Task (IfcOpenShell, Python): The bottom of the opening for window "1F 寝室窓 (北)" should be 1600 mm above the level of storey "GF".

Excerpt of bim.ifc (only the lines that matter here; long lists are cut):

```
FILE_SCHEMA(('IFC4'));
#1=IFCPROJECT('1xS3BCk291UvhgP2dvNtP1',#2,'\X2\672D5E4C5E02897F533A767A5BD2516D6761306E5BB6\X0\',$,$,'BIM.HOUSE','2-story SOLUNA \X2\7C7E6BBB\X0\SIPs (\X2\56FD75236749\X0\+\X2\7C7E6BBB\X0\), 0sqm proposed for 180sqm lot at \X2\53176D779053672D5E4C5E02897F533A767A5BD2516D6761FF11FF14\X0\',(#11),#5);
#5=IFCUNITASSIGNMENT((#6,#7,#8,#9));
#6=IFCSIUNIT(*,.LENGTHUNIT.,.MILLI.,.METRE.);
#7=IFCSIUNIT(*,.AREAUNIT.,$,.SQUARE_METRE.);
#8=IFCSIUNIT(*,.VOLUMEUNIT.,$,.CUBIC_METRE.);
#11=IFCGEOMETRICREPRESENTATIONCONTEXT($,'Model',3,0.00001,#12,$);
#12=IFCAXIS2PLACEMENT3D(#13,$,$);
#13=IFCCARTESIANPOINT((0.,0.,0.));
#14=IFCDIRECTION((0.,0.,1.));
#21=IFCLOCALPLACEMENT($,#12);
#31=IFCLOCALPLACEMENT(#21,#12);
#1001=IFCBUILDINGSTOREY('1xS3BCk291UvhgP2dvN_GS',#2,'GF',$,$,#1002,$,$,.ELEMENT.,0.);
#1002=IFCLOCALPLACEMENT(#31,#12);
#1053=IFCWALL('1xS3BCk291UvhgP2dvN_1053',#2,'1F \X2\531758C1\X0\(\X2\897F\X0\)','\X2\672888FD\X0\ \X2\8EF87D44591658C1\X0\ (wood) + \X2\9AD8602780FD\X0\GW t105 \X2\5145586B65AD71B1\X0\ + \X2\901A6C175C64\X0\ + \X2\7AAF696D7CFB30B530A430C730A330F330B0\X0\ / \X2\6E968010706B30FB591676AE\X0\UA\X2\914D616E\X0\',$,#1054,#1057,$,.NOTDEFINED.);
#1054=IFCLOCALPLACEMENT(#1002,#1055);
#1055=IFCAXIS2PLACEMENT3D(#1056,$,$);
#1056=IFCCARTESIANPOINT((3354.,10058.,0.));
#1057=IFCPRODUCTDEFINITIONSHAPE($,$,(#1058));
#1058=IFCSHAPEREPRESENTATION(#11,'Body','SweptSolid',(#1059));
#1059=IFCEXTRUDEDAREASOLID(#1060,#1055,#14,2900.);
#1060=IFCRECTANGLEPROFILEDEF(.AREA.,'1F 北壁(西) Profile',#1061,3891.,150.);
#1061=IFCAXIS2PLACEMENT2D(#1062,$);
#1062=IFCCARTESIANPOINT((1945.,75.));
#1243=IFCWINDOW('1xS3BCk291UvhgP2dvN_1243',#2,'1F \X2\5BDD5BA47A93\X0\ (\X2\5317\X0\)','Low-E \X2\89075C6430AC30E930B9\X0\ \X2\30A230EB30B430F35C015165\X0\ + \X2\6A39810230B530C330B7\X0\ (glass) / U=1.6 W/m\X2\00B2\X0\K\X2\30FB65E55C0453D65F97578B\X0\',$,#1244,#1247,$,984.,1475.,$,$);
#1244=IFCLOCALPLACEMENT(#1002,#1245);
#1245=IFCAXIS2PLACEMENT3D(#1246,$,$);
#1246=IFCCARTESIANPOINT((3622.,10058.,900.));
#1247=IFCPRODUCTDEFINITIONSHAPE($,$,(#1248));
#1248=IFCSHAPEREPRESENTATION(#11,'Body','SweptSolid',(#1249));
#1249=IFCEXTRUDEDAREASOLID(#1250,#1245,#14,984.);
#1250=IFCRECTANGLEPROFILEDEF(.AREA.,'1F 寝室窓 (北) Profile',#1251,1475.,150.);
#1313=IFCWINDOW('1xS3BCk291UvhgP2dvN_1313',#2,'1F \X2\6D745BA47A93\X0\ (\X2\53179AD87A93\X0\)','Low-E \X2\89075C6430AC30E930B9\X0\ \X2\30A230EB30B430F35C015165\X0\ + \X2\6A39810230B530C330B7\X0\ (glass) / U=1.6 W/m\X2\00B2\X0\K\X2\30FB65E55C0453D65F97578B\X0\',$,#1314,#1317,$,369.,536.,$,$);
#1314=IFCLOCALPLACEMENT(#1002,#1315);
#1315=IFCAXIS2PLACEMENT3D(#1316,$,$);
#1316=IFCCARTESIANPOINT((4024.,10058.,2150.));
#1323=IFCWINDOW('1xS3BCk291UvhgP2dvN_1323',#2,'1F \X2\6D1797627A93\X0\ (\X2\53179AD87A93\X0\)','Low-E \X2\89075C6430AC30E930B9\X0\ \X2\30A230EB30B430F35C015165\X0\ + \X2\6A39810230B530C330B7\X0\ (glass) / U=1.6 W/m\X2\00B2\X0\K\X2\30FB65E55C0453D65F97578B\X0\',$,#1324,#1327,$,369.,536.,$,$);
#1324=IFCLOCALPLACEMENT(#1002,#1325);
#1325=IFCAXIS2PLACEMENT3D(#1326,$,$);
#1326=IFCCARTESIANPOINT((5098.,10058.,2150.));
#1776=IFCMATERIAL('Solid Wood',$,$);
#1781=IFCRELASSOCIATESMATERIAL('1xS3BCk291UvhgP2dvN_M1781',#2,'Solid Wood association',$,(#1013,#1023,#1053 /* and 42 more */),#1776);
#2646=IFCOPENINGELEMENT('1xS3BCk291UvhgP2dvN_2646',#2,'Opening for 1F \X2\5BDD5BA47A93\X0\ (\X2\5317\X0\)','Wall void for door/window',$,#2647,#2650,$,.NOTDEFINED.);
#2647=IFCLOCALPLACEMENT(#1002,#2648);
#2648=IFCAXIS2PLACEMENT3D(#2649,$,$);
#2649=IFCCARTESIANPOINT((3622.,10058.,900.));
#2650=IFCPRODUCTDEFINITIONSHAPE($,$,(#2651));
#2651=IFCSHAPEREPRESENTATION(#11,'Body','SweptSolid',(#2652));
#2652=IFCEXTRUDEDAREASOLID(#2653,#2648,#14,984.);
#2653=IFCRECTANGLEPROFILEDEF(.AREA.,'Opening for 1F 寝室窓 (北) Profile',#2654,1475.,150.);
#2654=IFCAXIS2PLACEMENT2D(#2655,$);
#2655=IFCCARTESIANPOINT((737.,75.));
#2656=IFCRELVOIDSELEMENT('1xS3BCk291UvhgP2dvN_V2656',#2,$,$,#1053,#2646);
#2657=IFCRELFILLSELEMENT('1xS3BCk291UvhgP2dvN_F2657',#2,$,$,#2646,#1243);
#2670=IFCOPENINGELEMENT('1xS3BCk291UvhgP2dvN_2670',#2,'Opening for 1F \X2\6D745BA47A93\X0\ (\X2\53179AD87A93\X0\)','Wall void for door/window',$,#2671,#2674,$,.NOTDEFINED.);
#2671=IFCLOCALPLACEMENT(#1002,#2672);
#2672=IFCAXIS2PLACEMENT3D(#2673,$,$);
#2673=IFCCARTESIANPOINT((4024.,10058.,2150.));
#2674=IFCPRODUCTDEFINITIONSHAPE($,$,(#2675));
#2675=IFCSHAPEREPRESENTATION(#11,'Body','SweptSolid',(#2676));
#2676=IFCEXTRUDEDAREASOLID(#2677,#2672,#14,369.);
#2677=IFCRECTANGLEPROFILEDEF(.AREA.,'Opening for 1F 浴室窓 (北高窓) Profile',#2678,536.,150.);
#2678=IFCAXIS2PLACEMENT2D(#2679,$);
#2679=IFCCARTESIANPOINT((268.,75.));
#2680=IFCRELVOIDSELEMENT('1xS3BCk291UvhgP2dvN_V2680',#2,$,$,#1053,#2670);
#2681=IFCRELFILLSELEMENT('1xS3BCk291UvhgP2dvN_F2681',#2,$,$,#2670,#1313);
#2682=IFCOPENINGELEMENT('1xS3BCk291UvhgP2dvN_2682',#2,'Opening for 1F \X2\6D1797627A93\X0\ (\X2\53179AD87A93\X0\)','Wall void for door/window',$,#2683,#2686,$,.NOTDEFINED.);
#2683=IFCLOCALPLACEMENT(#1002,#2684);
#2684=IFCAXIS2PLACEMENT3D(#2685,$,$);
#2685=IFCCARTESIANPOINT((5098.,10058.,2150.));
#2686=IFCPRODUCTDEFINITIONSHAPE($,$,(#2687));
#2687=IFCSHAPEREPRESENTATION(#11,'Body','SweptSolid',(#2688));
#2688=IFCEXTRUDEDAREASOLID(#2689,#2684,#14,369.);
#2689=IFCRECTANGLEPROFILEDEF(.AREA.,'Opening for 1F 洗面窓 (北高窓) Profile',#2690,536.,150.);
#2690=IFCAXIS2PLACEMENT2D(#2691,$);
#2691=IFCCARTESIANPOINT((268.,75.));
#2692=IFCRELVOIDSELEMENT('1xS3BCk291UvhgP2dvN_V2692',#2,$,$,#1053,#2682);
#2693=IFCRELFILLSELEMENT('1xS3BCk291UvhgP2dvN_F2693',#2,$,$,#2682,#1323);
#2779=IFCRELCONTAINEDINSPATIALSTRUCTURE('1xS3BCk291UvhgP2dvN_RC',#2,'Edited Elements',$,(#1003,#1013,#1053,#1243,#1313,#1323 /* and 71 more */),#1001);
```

```python
import numpy as np
import ifcopenshell
import ifcopenshell.api.geometry
import ifcopenshell.geom
import ifcopenshell.util.element
import ifcopenshell.util.placement
import ifcopenshell.util.shape
import ifcopenshell.util.unit

model = ifcopenshell.open("bim.ifc")
unit_scale = ifcopenshell.util.unit.calculate_unit_scale(model)

window = model.by_id(1243)
opening = window.FillsVoids[0].RelatingOpeningElement
storey = ifcopenshell.util.element.get_container(window, ifc_class="IfcBuildingStorey")
level = ifcopenshell.util.placement.get_local_placement(storey.ObjectPlacement)[2, 3]

# The opening's origin need not be at the sill, so measure its lowest point.
shape = ifcopenshell.geom.create_shape(ifcopenshell.geom.settings(), opening)
bottom = ifcopenshell.util.shape.get_shape_bottom_elevation(shape, shape.geometry) / unit_scale
dz = level + 1600.0 - bottom

shift = np.array([0.0, 0.0, dz])
# The window is not placed relative to its opening, so move both.
for product in (opening, window):
    matrix = ifcopenshell.util.placement.get_local_placement(product.ObjectPlacement)
    matrix[:3, 3] += shift
    ifcopenshell.api.geometry.edit_object_placement(model, product=product, matrix=matrix, is_si=False)

print(f"moved by {dz * unit_scale:+.3f} m")

model.write("bim-out.ifc")
```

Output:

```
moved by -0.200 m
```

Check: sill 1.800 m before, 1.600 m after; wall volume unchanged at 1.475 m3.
